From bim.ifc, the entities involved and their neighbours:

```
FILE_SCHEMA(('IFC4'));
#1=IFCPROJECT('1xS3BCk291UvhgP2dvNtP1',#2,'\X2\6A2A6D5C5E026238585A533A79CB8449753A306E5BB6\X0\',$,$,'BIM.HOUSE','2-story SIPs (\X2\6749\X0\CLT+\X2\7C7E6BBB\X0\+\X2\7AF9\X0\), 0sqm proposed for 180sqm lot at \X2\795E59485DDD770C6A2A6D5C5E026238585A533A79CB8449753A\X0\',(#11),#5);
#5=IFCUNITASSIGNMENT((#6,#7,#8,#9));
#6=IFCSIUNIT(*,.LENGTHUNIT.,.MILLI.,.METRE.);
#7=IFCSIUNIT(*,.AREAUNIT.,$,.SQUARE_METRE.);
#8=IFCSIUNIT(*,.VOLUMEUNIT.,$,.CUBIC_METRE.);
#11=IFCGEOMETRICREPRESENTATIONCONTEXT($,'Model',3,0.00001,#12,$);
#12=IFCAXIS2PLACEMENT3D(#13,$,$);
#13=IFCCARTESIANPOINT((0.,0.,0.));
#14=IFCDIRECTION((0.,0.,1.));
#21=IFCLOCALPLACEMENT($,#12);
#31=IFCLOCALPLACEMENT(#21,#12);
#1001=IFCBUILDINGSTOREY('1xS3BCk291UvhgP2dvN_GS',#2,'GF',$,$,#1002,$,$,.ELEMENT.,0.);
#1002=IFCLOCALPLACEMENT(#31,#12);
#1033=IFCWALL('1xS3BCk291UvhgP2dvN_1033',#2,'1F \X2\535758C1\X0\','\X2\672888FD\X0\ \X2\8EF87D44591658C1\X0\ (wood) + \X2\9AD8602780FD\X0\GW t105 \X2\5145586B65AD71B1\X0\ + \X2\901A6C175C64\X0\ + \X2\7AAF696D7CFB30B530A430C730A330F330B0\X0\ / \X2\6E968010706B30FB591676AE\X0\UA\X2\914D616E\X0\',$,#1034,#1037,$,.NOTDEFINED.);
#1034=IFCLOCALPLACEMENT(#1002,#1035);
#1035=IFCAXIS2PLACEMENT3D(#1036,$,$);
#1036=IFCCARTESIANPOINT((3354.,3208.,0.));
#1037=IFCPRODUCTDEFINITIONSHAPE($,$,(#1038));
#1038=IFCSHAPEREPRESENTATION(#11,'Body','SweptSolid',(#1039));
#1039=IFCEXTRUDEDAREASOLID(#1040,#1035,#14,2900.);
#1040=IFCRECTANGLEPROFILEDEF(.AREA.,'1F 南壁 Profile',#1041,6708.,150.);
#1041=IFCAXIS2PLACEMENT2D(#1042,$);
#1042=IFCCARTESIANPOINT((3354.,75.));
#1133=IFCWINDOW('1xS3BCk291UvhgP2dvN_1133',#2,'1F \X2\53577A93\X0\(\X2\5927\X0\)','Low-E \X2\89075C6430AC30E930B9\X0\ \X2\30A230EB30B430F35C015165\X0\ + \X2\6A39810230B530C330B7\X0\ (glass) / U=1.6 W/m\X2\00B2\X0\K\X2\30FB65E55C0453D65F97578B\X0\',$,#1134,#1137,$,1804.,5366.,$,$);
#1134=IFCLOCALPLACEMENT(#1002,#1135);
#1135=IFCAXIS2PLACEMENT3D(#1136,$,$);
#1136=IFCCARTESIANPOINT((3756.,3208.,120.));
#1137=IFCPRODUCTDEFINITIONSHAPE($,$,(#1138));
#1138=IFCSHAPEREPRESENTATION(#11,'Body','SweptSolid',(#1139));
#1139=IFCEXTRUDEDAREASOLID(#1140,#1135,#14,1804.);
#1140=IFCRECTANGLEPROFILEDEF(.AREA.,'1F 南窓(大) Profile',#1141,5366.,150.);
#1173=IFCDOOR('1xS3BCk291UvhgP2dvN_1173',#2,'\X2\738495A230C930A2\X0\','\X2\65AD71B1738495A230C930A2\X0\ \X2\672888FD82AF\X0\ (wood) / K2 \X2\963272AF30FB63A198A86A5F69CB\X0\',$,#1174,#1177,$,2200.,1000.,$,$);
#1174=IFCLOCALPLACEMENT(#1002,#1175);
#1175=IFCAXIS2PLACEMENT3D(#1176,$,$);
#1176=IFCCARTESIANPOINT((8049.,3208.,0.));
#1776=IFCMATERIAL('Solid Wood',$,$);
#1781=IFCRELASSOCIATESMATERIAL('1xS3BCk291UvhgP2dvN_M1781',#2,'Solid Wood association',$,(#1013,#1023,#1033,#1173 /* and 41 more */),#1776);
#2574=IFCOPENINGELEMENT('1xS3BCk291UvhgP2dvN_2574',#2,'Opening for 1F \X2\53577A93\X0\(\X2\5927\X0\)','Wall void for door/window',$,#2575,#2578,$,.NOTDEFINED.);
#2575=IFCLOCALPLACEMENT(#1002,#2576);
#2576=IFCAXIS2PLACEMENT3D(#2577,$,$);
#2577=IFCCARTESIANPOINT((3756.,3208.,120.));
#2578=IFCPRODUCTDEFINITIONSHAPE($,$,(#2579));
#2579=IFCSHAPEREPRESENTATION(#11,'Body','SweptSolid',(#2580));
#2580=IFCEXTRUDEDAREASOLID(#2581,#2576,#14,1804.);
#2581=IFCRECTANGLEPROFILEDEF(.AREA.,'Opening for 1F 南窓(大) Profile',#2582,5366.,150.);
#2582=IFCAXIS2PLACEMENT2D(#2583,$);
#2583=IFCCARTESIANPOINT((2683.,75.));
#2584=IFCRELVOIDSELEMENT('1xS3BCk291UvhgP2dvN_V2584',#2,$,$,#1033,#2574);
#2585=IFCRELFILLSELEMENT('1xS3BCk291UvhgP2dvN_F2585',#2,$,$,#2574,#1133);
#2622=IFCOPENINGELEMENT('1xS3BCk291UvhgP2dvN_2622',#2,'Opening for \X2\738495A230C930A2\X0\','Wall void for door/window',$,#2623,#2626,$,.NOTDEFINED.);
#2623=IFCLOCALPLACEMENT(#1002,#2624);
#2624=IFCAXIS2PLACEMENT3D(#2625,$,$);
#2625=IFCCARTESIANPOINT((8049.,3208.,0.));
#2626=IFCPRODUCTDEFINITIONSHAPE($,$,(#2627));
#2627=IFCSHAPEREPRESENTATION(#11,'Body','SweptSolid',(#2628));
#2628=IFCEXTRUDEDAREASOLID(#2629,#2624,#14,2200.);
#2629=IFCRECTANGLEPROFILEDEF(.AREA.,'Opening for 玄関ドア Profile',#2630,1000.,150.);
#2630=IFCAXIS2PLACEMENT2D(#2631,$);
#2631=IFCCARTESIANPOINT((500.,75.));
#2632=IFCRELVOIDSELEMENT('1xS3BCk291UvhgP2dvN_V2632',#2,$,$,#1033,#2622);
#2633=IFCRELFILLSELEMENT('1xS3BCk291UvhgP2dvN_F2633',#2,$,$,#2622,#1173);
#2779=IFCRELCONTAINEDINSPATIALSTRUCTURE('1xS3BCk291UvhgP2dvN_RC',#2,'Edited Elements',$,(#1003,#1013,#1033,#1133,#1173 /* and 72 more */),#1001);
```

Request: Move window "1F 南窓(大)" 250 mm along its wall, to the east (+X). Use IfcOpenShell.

```python
import ifcopenshell
import ifcopenshell.api.geometry
import ifcopenshell.util.placement

model = ifcopenshell.open("bim.ifc")

window = model.by_id(1133)
opening = window.FillsVoids[0].RelatingOpeningElement
wall = opening.VoidsElements[0].RelatingBuildingElement

wall_matrix = ifcopenshell.util.placement.get_local_placement(wall.ObjectPlacement)
shift = wall_matrix[:3, 0] * 250.0
before = ifcopenshell.util.placement.get_local_placement(window.ObjectPlacement)[:3, 3].copy()

# The window is not placed relative to its opening, so move both.
for product in (opening, window):
    matrix = ifcopenshell.util.placement.get_local_placement(product.ObjectPlacement)
    matrix[:3, 3] += shift
    ifcopenshell.api.geometry.edit_object_placement(model, product=product, matrix=matrix, is_si=False)

after = ifcopenshell.util.placement.get_local_placement(window.ObjectPlacement)[:3, 3]
print("window moved by", (after - before).round(3) + 0.0)

model.write("bim_v2.ifc")
```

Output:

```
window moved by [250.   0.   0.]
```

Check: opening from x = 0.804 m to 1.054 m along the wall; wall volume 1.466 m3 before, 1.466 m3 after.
